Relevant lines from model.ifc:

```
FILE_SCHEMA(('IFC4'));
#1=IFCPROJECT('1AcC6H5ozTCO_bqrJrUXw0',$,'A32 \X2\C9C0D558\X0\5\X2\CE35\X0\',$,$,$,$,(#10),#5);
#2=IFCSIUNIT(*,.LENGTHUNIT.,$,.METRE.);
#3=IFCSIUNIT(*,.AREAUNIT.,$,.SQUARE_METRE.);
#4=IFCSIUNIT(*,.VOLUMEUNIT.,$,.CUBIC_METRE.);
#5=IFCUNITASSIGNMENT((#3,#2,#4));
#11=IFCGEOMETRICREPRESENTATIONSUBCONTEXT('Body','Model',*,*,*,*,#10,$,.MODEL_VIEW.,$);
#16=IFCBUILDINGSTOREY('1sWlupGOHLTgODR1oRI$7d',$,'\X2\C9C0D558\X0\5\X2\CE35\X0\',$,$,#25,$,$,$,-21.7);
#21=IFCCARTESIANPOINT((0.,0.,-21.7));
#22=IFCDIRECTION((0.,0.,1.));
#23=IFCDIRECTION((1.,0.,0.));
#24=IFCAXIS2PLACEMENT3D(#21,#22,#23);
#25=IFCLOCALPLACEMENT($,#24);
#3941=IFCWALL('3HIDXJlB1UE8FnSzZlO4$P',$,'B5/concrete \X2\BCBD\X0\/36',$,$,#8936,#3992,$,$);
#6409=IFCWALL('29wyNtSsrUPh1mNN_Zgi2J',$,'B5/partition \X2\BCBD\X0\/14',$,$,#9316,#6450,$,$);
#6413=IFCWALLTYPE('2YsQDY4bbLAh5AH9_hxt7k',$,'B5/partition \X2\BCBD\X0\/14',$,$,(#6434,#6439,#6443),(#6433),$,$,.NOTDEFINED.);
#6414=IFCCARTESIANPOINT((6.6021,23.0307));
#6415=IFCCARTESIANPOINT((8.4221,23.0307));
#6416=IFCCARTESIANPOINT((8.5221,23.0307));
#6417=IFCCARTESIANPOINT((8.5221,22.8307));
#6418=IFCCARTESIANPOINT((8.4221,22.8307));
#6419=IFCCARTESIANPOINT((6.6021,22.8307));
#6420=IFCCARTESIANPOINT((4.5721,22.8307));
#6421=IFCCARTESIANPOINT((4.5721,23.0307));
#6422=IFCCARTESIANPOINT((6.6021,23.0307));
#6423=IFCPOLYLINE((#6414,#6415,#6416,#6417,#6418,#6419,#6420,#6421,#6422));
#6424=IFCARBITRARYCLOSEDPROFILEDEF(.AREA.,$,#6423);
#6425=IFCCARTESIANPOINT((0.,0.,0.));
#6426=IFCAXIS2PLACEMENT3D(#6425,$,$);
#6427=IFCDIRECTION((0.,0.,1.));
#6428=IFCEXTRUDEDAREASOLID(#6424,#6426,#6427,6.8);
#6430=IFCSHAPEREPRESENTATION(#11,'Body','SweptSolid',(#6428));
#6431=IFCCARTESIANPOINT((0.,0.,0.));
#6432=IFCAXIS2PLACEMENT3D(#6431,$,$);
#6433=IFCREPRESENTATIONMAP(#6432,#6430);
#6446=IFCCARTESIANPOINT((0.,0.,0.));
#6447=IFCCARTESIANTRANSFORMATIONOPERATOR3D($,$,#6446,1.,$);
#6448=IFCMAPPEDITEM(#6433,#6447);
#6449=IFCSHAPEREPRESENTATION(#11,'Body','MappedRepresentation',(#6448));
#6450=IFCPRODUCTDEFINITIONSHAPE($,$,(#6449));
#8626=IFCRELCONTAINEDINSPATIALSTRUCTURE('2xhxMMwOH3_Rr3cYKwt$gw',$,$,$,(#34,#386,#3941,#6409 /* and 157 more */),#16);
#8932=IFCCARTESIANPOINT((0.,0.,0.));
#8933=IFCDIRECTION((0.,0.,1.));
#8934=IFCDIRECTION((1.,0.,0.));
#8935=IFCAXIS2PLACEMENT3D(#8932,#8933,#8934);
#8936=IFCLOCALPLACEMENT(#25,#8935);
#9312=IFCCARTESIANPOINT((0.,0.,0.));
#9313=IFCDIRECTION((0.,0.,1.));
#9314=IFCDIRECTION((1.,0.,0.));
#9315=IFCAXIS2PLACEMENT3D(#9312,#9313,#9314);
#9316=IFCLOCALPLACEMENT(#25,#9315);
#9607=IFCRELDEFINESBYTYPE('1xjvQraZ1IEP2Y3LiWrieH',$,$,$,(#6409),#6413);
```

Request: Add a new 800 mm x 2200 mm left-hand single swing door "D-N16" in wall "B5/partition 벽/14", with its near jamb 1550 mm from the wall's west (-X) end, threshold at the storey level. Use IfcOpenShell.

```python
import numpy as np
import ifcopenshell
import ifcopenshell.api.feature
import ifcopenshell.api.geometry
import ifcopenshell.api.root
import ifcopenshell.api.spatial
import ifcopenshell.geom
import ifcopenshell.util.element
import ifcopenshell.util.placement
import ifcopenshell.util.representation
import ifcopenshell.util.shape
import ifcopenshell.util.unit

model = ifcopenshell.open("model.ifc")
unit_scale = ifcopenshell.util.unit.calculate_unit_scale(model)
settings = ifcopenshell.geom.settings()


def volume(element):
    """Net volume in cubic metres, openings subtracted."""
    shape = ifcopenshell.geom.create_shape(settings, element)
    return ifcopenshell.util.shape.get_volume(shape.geometry)


wall = model.by_guid("29wyNtSsrUPh1mNN_Zgi2J")
storey = ifcopenshell.util.element.get_container(wall, ifc_class="IfcBuildingStorey")
context = ifcopenshell.util.representation.get_context(model, "Model", "Body", "MODEL_VIEW")
before = volume(wall)

width, height, from_end, sill = 0.8, 2.2, 1.55, 0.0  # metres

# The wall runs along its own X axis, and the end named is its -X end.
wall_shape = ifcopenshell.geom.create_shape(settings, wall)
x, y, z = ifcopenshell.util.shape.get_vertices(wall_shape.geometry).T
start = x.min() + from_end
face, thickness = float(y.min()), float(y.max() - y.min())
wall_matrix = ifcopenshell.util.placement.get_local_placement(wall.ObjectPlacement)
level = ifcopenshell.util.placement.get_local_placement(storey.ObjectPlacement)[2, 3]


def in_wall(x, y):
    """Placement at x, y metres in the wall's axes, at sill height."""
    matrix = wall_matrix.copy()
    matrix[:, 3] = wall_matrix @ np.array([x / unit_scale, y / unit_scale, 0.0, 1.0])
    matrix[2, 3] = level + sill / unit_scale
    return matrix


# Opening: a box that overshoots both wall faces by 50 mm.
opening = ifcopenshell.api.root.create_entity(model, ifc_class="IfcOpeningElement", predefined_type="OPENING")
box = ifcopenshell.api.geometry.add_wall_representation(
    model, context=context, length=width, height=height, thickness=thickness + 0.1
)
ifcopenshell.api.geometry.assign_representation(model, product=opening, representation=box)
ifcopenshell.api.geometry.edit_object_placement(model, product=opening, matrix=in_wall(start, face - 0.05), is_si=False)
ifcopenshell.api.feature.add_feature(model, feature=opening, element=wall)

door = ifcopenshell.api.root.create_entity(model, ifc_class="IfcDoor", name="D-N16", predefined_type="DOOR")
door.OverallWidth, door.OverallHeight = width / unit_scale, height / unit_scale
door.OperationType = "SINGLE_SWING_LEFT"
body = ifcopenshell.api.geometry.add_door_representation(
    model,
    context=context,
    overall_width=door.OverallWidth,
    overall_height=door.OverallHeight,
    operation_type="SINGLE_SWING_LEFT",
    lining_properties={"LiningDepth": thickness / unit_scale, "ThresholdDepth": thickness / unit_scale},
)
ifcopenshell.api.geometry.assign_representation(model, product=door, representation=body)
ifcopenshell.api.spatial.assign_container(model, products=[door], relating_structure=storey)
ifcopenshell.api.feature.add_filling(model, opening=opening, element=door)

# The lining spans the wall, so the door starts at the wall face.
ifcopenshell.api.geometry.edit_object_placement(model, product=door, matrix=in_wall(start, face), is_si=False)

after = volume(wall)

print(f"wall volume {before:.3f} -> {after:.3f} m3")

model.write("model_v2.ifc")
```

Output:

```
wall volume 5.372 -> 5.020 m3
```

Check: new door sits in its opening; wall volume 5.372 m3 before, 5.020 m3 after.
